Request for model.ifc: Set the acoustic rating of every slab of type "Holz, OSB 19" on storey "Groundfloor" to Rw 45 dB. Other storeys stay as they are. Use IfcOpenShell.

First a look at what the model holds.

```python
import ifcopenshell
import ifcopenshell.util.element

model = ifcopenshell.open("model.ifc")
print(model.schema)
storey = next(s for s in model.by_type("IfcBuildingStorey") if s.Name == "Groundfloor")
slabs = [e for e in ifcopenshell.util.element.get_decomposition(storey) if e.is_a("IfcSlab")]
seen = {}
for e in slabs:
    element_type = ifcopenshell.util.element.get_type(e)
    key = (element_type.Name if element_type != e and element_type else None, ifcopenshell.util.element.get_pset(e, "Pset_SlabCommon", "AcousticRating"))
    seen[key] = seen.get(key, 0) + 1
for (name, value), count in sorted(seen.items(), key=str):
    print(count, "x", name, "|", value)
```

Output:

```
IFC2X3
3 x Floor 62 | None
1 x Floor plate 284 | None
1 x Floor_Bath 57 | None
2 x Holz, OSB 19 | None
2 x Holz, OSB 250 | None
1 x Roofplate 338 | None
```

```python
import ifcopenshell
import ifcopenshell.api.pset
import ifcopenshell.util.element

model = ifcopenshell.open("model.ifc")

storey = next(s for s in model.by_type("IfcBuildingStorey") if s.Name == "Groundfloor")
slabs = [e for e in ifcopenshell.util.element.get_decomposition(storey) if e.is_a("IfcSlab")]

count = 0
for e in slabs:
    element_type = ifcopenshell.util.element.get_type(e)
    if element_type in (None, e) or element_type.Name != "Holz, OSB 19":
        continue
    # add_pset returns the element's existing set when there is one.
    pset = ifcopenshell.api.pset.add_pset(model, product=e, name="Pset_SlabCommon")
    ifcopenshell.api.pset.edit_pset(model, pset=pset, properties={"AcousticRating": "Rw 45 dB"})
    count += 1

print(count, "slabs updated")

model.write("model-out.ifc")
```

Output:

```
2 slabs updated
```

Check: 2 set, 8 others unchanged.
